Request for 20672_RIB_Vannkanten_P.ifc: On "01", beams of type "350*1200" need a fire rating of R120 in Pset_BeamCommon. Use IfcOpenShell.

First a look at what the model holds.

```python
import ifcopenshell
import ifcopenshell.util.element

model = ifcopenshell.open("20672_RIB_Vannkanten_P.ifc")
print(model.schema)
storey = next(s for s in model.by_type("IfcBuildingStorey") if s.Name == "01")
beams = [e for e in ifcopenshell.util.element.get_decomposition(storey) if e.is_a("IfcBeam")]
seen = {}
for e in beams:
    element_type = ifcopenshell.util.element.get_type(e)
    key = (element_type.Name if element_type != e and element_type else None, ifcopenshell.util.element.get_pset(e, "Pset_BeamCommon", "FireRating"))
    seen[key] = seen.get(key, 0) + 1
for (name, value), count in sorted(seen.items(), key=str):
    print(count, "x", name, "|", value)
```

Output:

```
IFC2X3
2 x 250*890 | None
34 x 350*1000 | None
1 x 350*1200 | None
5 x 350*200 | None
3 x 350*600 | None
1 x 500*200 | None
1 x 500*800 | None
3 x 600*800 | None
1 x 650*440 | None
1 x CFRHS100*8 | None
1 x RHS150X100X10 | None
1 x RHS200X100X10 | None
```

```python
import ifcopenshell
import ifcopenshell.api.pset
import ifcopenshell.util.element

model = ifcopenshell.open("20672_RIB_Vannkanten_P.ifc")

storey = next(s for s in model.by_type("IfcBuildingStorey") if s.Name == "01")
beams = [e for e in ifcopenshell.util.element.get_decomposition(storey) if e.is_a("IfcBeam")]

count = 0
for e in beams:
    element_type = ifcopenshell.util.element.get_type(e)
    if element_type in (None, e) or element_type.Name != "350*1200":
        continue
    # add_pset returns the element's existing set when there is one.
    pset = ifcopenshell.api.pset.add_pset(model, product=e, name="Pset_BeamCommon")
    ifcopenshell.api.pset.edit_pset(model, pset=pset, properties={"FireRating": "R120"})
    count += 1

print(count, "beams updated")

model.write("20672_RIB_Vannkanten_P_updated.ifc")
```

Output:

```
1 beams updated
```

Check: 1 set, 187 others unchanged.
